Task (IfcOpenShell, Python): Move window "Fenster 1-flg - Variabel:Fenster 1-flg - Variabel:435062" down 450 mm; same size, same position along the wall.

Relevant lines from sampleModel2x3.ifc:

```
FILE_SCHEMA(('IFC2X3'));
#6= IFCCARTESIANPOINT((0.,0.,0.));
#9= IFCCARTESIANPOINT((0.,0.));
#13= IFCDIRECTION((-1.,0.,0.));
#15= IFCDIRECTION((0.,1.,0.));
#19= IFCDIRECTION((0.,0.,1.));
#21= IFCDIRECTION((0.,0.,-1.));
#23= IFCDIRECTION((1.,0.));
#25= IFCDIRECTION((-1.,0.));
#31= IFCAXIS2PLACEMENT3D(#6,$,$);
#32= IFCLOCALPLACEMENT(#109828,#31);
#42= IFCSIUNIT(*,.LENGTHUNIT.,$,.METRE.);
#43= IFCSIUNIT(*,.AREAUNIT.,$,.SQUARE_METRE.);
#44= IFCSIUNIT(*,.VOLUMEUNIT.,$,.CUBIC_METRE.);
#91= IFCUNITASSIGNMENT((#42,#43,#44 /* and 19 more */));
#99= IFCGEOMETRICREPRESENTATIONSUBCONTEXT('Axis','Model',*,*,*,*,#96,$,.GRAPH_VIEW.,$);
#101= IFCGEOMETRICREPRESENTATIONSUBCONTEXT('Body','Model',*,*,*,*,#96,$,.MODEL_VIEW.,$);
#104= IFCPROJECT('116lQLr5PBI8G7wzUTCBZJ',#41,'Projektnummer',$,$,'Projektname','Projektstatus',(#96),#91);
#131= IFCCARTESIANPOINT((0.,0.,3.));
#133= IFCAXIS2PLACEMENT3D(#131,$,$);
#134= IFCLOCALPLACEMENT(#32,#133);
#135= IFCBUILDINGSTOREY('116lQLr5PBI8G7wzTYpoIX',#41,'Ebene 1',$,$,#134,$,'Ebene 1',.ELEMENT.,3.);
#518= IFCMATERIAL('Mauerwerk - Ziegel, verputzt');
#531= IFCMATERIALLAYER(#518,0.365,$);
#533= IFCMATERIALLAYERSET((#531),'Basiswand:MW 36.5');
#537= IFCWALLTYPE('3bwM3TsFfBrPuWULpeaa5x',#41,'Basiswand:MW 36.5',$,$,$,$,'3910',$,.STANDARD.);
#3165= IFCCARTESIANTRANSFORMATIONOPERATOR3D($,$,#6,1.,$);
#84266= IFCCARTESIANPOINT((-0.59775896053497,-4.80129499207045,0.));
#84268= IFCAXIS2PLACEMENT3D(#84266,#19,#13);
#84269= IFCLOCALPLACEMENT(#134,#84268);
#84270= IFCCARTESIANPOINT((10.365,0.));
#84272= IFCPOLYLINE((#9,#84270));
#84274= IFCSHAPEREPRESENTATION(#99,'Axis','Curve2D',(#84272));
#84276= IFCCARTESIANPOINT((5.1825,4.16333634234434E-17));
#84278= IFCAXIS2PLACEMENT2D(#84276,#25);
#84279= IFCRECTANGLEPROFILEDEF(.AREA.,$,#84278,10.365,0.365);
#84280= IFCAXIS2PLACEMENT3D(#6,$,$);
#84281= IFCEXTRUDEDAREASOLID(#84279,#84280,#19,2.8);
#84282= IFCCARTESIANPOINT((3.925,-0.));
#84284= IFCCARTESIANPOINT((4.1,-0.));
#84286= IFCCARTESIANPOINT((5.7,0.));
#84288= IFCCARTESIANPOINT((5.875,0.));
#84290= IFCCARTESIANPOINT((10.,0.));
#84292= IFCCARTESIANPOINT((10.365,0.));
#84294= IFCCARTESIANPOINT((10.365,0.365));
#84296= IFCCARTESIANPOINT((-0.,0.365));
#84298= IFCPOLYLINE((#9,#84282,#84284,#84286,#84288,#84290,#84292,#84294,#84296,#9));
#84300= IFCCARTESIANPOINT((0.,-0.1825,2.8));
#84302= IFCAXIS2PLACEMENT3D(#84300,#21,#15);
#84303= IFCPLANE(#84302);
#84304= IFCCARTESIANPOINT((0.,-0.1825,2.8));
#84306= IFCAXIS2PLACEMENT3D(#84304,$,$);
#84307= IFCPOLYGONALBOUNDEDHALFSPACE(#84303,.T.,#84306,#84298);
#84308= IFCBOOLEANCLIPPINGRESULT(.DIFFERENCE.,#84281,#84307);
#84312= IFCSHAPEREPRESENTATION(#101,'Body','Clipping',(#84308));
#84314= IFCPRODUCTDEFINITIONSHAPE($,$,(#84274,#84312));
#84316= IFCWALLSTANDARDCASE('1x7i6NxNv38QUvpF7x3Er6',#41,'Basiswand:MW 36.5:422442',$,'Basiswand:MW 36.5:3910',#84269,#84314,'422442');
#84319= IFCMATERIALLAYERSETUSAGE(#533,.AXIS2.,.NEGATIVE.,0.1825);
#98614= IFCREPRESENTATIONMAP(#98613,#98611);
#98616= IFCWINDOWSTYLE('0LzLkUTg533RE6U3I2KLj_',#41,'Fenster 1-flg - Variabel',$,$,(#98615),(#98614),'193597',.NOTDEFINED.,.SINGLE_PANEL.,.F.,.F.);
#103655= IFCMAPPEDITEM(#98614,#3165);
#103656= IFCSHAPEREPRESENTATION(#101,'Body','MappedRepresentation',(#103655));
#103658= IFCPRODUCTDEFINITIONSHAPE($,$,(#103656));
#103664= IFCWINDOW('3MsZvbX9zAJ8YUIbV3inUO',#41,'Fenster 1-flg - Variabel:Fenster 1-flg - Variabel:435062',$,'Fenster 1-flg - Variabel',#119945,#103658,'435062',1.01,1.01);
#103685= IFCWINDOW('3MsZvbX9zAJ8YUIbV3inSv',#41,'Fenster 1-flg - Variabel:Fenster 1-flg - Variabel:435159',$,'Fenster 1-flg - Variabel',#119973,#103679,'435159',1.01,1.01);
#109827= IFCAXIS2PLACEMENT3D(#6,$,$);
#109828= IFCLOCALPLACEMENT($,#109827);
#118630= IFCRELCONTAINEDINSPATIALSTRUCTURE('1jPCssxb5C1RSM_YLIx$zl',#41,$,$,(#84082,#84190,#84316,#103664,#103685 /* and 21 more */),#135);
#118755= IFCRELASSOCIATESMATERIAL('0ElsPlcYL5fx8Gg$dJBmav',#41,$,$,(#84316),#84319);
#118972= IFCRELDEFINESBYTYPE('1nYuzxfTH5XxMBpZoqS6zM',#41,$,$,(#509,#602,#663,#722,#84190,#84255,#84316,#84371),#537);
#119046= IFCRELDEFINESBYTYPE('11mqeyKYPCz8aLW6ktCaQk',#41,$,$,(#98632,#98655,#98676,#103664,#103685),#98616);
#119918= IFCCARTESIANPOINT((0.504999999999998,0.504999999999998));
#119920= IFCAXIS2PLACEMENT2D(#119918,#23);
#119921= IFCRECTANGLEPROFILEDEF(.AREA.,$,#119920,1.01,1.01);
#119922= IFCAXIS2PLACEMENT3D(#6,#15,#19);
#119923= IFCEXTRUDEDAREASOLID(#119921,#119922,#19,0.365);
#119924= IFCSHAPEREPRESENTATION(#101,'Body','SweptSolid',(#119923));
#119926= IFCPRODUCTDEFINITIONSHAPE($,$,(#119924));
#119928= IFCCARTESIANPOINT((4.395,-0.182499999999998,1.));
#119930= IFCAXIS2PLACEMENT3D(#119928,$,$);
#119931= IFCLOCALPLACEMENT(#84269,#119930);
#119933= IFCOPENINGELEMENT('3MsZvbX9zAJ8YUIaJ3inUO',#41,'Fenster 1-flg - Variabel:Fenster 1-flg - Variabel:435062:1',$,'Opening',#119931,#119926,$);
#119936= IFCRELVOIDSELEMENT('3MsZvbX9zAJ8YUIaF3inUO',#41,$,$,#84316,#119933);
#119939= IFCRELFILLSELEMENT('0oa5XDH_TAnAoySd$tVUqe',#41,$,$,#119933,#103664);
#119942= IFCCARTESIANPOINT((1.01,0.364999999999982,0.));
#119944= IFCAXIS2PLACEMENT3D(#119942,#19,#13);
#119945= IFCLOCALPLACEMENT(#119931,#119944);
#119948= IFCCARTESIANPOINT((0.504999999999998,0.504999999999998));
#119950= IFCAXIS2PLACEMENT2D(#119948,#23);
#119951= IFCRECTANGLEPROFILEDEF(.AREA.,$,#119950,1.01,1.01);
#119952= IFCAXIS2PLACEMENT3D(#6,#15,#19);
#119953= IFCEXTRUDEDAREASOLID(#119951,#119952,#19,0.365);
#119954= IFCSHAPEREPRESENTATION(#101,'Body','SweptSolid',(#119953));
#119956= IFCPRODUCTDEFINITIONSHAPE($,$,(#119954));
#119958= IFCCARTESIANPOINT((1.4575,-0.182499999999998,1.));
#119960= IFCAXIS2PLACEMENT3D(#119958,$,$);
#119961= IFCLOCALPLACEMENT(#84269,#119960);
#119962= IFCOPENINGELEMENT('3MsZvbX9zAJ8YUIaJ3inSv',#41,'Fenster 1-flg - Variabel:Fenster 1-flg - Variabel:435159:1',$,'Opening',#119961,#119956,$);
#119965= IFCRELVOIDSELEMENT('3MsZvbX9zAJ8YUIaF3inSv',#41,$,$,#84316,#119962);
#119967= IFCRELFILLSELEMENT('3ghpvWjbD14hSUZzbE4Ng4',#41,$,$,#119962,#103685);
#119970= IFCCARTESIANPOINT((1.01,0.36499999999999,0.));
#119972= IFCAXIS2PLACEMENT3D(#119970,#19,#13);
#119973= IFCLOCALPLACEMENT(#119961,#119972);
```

```python
import numpy as np
import ifcopenshell
import ifcopenshell.api.geometry
import ifcopenshell.util.placement
import ifcopenshell.util.unit

model = ifcopenshell.open("sampleModel2x3.ifc")
unit_scale = ifcopenshell.util.unit.calculate_unit_scale(model)

window = model.by_guid("3MsZvbX9zAJ8YUIbV3inUO")
opening = window.FillsVoids[0].RelatingOpeningElement
dz = -0.45 / unit_scale

shift = np.array([0.0, 0.0, dz])
# The window is placed relative to its opening, so it follows when the opening moves.
matrix = ifcopenshell.util.placement.get_local_placement(opening.ObjectPlacement)
matrix[:3, 3] += shift
ifcopenshell.api.geometry.edit_object_placement(
    model, product=opening, matrix=matrix, is_si=False, should_transform_children=True
)

print(f"moved by {dz * unit_scale:+.3f} m")

model.write("sampleModel2x3_rev.ifc")
```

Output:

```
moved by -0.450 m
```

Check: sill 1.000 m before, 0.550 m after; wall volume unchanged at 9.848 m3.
